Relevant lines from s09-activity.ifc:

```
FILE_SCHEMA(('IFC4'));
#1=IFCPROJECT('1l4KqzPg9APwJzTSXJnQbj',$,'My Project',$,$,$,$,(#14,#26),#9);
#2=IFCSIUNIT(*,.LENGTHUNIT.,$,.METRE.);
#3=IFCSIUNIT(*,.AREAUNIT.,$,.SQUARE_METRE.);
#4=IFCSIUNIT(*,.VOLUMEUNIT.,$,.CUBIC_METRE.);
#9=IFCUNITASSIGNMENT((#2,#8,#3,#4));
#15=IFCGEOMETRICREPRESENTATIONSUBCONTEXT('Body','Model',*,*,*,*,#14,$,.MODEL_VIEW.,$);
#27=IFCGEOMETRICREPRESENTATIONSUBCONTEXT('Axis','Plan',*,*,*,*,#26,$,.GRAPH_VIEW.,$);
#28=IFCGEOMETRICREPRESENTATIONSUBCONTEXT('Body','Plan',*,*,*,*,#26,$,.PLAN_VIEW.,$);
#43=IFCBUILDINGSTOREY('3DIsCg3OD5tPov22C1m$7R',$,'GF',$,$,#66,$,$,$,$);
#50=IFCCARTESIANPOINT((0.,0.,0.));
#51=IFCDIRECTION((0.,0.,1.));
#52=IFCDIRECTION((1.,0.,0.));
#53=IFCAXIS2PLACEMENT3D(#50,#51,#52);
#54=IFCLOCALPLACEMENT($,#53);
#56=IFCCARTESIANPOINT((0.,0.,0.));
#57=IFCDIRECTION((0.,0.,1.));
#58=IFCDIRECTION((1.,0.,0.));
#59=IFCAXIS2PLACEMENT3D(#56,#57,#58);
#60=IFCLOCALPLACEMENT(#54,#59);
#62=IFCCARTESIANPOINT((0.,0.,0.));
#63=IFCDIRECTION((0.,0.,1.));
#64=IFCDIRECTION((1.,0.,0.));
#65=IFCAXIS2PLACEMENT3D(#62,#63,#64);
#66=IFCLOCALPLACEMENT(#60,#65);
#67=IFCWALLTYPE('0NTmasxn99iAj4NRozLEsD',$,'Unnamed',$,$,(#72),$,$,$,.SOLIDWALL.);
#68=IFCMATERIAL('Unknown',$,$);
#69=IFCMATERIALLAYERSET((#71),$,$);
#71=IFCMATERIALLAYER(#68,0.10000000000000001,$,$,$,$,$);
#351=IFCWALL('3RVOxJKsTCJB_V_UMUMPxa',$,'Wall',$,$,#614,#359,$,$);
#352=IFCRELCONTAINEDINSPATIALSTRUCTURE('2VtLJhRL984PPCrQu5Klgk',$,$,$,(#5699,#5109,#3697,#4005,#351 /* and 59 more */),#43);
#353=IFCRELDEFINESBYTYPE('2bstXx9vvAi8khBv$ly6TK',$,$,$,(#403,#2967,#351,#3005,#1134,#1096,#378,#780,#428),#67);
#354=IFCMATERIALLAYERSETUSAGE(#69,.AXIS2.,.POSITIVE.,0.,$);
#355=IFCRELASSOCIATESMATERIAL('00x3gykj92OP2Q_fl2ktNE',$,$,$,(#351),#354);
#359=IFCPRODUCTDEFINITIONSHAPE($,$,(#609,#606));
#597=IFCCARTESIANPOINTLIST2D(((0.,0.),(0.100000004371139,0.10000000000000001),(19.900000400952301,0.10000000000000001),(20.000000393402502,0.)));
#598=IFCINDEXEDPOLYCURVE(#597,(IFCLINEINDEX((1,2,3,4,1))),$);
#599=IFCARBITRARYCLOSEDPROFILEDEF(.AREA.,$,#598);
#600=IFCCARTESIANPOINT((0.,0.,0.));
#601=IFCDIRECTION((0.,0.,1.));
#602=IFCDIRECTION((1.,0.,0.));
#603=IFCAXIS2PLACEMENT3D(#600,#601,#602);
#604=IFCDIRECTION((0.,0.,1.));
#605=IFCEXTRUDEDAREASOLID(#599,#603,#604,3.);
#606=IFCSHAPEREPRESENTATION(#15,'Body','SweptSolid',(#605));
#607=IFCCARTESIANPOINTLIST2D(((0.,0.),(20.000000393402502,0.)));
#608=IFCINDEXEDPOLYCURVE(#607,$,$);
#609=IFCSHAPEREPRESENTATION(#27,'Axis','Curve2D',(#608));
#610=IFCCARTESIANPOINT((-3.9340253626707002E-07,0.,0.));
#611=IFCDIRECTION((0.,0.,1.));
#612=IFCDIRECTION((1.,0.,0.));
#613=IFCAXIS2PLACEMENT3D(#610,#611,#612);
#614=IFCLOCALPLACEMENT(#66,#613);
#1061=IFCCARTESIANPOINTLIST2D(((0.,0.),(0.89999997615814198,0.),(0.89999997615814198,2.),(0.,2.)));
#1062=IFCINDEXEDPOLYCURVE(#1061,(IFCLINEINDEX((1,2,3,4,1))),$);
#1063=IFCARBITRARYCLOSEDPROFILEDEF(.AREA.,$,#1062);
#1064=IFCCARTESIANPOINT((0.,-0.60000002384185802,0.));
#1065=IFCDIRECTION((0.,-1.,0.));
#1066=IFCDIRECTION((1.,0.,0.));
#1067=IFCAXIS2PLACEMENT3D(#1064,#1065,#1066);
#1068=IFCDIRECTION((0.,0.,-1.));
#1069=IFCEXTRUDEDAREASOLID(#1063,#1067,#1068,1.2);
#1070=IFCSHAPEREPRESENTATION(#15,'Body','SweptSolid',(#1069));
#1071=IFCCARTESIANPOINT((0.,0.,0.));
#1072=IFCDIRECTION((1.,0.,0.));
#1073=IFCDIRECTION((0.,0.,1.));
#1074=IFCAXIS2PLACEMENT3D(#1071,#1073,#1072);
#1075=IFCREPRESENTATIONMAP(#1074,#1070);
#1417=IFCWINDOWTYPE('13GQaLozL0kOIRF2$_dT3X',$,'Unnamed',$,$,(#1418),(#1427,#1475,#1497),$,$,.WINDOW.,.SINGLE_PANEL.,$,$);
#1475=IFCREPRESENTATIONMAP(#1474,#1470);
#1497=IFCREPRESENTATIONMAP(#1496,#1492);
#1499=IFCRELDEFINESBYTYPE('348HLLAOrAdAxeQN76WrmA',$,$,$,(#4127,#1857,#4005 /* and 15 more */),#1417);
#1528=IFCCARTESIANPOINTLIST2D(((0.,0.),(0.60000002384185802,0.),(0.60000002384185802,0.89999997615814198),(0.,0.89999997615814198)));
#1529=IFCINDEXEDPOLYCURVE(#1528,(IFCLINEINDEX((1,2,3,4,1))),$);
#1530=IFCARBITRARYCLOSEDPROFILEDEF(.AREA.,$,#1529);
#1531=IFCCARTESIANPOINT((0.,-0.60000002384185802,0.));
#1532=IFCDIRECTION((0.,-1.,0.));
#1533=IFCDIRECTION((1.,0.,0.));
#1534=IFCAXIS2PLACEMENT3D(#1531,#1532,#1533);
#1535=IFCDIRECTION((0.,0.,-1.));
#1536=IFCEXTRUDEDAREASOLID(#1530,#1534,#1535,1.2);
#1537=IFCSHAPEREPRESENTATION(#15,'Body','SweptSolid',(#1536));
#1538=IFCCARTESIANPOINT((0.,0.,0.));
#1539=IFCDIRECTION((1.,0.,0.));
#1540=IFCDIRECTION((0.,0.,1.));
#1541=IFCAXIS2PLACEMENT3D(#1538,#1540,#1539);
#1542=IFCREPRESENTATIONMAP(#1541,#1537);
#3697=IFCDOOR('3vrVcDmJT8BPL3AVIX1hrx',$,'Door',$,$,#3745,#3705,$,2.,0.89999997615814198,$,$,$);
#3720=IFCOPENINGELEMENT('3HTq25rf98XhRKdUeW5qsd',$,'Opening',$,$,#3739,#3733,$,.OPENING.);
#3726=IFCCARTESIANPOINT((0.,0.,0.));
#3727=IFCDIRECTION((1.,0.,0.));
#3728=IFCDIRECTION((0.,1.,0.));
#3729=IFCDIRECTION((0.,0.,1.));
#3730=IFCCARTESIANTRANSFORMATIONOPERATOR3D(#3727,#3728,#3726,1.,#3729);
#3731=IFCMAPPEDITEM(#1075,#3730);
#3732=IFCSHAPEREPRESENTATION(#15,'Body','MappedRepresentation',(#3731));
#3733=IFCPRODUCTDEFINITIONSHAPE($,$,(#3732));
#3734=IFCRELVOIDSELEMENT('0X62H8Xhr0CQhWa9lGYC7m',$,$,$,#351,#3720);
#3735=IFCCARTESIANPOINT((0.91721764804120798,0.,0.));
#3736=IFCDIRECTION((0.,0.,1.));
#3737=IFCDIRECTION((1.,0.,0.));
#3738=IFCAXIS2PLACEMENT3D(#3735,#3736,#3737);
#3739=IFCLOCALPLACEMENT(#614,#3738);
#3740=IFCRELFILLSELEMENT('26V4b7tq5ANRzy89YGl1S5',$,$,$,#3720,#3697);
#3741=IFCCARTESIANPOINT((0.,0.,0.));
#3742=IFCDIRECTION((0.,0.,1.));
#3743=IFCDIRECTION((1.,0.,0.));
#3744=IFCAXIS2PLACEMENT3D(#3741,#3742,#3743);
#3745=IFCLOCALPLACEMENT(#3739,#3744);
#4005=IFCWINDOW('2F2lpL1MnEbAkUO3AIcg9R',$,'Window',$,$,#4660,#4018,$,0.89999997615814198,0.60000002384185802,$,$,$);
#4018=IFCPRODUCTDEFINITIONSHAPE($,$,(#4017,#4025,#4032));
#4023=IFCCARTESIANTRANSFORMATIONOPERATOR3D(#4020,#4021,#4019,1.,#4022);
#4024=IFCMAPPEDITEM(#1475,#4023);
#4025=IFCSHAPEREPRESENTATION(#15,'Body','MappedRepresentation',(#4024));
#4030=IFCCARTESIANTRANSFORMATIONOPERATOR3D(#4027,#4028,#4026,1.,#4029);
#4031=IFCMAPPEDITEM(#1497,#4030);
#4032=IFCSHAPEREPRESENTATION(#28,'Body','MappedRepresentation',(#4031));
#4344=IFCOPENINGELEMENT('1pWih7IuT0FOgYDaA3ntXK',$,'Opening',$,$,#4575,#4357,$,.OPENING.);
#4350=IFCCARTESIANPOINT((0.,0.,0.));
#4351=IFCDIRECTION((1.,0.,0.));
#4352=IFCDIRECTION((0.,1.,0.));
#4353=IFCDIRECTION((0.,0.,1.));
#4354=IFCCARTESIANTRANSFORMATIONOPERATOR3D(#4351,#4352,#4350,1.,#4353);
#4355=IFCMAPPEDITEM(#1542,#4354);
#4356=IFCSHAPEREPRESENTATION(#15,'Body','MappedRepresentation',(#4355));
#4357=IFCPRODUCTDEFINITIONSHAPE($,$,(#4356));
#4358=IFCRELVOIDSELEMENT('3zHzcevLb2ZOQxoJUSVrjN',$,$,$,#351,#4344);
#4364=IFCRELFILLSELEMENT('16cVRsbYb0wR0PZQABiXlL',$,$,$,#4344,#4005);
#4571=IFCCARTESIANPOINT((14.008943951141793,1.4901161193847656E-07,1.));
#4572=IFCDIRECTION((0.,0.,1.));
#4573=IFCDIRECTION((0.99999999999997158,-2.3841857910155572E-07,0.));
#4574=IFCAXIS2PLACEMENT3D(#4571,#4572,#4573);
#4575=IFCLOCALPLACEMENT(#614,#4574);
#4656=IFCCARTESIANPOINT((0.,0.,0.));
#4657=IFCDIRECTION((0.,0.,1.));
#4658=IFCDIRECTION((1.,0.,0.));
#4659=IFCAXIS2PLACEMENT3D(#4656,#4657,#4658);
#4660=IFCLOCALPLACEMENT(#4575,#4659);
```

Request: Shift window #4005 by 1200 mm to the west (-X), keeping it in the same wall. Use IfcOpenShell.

```python
import ifcopenshell
import ifcopenshell.api.geometry
import ifcopenshell.util.placement
import ifcopenshell.util.unit

model = ifcopenshell.open("s09-activity.ifc")
unit_scale = ifcopenshell.util.unit.calculate_unit_scale(model)

window = model.by_id(4005)
opening = window.FillsVoids[0].RelatingOpeningElement
wall = opening.VoidsElements[0].RelatingBuildingElement

wall_matrix = ifcopenshell.util.placement.get_local_placement(wall.ObjectPlacement)
shift = wall_matrix[:3, 0] * -1.2 / unit_scale
before = ifcopenshell.util.placement.get_local_placement(window.ObjectPlacement)[:3, 3].copy()

# The window is placed relative to its opening, so it follows when the opening moves.
matrix = ifcopenshell.util.placement.get_local_placement(opening.ObjectPlacement)
matrix[:3, 3] += shift
ifcopenshell.api.geometry.edit_object_placement(
    model, product=opening, matrix=matrix, is_si=False, should_transform_children=True
)

after = ifcopenshell.util.placement.get_local_placement(window.ObjectPlacement)[:3, 3]
print("window moved by", (after - before).round(3) + 0.0)

model.write("s09-activity-out.ifc")
```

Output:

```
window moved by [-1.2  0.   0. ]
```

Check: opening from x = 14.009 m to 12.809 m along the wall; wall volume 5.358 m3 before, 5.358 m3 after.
